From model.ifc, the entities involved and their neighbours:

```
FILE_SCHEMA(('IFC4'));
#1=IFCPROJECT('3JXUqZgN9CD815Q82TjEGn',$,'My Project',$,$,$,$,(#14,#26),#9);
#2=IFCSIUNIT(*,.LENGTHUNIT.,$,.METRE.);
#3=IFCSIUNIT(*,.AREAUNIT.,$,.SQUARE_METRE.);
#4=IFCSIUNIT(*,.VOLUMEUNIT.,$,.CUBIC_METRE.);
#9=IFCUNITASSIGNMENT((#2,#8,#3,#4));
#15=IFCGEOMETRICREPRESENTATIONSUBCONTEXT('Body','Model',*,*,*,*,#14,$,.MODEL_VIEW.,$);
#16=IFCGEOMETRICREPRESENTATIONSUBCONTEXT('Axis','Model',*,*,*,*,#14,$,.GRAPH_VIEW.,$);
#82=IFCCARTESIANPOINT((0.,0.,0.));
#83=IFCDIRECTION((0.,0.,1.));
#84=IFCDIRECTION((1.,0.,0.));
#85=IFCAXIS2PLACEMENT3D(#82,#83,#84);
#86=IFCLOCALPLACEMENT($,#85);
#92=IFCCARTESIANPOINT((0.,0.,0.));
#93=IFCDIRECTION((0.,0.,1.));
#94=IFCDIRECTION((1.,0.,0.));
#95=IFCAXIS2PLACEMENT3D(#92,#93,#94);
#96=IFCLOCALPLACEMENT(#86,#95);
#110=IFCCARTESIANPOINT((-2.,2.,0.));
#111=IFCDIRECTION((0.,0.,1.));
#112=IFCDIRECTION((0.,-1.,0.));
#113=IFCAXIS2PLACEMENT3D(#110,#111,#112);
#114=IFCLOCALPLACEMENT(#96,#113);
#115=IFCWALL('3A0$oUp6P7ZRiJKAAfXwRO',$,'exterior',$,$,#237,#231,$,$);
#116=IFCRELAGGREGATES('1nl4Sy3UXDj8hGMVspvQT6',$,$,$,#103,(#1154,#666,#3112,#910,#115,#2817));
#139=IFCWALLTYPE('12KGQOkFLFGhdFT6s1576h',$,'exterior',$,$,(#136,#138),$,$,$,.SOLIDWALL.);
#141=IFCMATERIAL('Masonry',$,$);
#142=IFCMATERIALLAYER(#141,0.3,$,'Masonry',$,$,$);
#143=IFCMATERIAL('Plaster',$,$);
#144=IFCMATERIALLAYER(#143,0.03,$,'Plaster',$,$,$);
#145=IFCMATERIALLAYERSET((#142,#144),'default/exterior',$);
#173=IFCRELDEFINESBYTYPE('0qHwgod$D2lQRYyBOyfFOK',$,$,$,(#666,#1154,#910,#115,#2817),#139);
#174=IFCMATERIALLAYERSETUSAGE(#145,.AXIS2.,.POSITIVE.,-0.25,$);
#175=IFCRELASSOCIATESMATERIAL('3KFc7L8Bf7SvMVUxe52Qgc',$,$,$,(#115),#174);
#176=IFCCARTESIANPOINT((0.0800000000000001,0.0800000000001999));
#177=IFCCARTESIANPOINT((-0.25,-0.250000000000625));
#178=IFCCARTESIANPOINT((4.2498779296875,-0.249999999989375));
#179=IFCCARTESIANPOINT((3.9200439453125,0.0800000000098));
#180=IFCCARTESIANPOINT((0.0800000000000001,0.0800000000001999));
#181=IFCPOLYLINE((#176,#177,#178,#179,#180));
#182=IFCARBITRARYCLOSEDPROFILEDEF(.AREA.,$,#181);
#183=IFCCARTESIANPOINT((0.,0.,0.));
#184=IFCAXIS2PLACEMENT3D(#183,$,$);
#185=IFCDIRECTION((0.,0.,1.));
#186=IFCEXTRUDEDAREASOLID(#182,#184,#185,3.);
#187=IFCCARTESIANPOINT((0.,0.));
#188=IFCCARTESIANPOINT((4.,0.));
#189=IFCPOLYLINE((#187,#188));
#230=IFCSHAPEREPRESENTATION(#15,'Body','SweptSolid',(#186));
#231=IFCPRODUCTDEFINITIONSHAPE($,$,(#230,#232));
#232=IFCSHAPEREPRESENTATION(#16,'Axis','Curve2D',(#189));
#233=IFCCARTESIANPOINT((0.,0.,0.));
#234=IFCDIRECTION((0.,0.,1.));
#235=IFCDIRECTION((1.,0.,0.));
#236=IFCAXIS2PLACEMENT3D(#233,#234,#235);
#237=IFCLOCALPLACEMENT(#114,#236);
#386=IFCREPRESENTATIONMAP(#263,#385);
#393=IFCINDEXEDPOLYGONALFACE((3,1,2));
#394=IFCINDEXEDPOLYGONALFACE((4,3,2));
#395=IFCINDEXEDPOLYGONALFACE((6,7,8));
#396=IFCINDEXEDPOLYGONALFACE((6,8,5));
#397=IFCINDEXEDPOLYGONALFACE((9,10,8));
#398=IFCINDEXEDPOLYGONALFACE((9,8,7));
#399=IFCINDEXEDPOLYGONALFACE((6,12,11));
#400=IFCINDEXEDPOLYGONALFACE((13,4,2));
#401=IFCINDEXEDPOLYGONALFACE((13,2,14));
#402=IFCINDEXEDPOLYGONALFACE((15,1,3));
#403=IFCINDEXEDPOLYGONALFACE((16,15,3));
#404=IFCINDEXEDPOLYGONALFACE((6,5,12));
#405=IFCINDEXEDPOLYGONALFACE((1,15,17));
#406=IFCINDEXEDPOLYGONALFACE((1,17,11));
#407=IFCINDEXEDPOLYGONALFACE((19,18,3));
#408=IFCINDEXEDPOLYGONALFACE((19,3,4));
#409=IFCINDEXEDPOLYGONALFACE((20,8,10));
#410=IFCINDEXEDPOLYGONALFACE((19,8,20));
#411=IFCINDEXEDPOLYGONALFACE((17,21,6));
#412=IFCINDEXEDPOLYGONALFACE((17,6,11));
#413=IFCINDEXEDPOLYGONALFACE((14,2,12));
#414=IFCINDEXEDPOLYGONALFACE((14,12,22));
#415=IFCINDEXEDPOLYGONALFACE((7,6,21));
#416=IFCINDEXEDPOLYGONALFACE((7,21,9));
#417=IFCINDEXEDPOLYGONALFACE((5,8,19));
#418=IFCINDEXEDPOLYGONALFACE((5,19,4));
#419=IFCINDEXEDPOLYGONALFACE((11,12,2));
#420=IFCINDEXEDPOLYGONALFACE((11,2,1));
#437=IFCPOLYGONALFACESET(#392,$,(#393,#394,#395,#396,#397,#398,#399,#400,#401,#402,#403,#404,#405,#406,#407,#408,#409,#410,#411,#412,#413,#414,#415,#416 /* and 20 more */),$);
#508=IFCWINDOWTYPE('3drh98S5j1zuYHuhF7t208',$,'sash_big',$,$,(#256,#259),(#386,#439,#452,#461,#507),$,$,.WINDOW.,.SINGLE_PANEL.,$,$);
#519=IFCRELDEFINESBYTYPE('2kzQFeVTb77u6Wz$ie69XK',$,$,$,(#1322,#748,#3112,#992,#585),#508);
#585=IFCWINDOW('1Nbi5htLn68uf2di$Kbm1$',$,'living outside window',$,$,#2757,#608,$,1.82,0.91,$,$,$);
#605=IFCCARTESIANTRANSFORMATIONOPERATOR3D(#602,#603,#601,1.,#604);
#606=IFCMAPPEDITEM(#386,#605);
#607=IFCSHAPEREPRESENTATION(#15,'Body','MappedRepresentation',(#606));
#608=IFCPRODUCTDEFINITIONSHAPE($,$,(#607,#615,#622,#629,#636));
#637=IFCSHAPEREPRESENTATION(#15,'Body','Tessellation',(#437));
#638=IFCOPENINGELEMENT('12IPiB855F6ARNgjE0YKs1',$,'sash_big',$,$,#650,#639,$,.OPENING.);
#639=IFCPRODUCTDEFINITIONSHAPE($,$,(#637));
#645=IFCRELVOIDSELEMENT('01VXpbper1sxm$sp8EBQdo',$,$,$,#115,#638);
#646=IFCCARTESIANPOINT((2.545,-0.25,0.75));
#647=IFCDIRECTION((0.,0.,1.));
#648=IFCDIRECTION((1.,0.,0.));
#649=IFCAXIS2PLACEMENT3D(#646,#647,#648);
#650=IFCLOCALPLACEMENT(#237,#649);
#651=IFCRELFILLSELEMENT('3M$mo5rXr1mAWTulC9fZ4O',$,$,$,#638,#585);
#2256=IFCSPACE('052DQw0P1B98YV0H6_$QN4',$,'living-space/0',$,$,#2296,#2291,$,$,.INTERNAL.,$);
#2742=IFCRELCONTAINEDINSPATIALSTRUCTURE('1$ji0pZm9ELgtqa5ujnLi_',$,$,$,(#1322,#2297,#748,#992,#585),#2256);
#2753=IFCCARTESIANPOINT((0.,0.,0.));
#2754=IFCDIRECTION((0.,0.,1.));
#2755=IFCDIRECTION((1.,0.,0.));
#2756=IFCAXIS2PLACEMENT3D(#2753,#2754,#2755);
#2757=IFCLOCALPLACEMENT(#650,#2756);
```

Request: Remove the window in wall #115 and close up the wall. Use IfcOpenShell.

```python
import ifcopenshell
import ifcopenshell.api.feature
import ifcopenshell.api.root
import ifcopenshell.geom
import ifcopenshell.util.shape

model = ifcopenshell.open("model.ifc")
settings = ifcopenshell.geom.settings()


def volume(element):
    """Net volume in cubic metres, openings subtracted."""
    shape = ifcopenshell.geom.create_shape(settings, element)
    return ifcopenshell.util.shape.get_volume(shape.geometry)


window = model.by_guid("1Nbi5htLn68uf2di$Kbm1$")
opening = window.FillsVoids[0].RelatingOpeningElement
wall = opening.VoidsElements[0].RelatingBuildingElement
before = volume(wall)

ifcopenshell.api.root.remove_product(model, product=window)
ifcopenshell.api.feature.remove_feature(model, feature=opening)

after = volume(wall)

print(f"wall volume {before:.3f} -> {after:.3f} m3")

model.write("model_rev.ifc")
```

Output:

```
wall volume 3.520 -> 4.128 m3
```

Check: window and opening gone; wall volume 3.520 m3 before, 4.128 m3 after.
